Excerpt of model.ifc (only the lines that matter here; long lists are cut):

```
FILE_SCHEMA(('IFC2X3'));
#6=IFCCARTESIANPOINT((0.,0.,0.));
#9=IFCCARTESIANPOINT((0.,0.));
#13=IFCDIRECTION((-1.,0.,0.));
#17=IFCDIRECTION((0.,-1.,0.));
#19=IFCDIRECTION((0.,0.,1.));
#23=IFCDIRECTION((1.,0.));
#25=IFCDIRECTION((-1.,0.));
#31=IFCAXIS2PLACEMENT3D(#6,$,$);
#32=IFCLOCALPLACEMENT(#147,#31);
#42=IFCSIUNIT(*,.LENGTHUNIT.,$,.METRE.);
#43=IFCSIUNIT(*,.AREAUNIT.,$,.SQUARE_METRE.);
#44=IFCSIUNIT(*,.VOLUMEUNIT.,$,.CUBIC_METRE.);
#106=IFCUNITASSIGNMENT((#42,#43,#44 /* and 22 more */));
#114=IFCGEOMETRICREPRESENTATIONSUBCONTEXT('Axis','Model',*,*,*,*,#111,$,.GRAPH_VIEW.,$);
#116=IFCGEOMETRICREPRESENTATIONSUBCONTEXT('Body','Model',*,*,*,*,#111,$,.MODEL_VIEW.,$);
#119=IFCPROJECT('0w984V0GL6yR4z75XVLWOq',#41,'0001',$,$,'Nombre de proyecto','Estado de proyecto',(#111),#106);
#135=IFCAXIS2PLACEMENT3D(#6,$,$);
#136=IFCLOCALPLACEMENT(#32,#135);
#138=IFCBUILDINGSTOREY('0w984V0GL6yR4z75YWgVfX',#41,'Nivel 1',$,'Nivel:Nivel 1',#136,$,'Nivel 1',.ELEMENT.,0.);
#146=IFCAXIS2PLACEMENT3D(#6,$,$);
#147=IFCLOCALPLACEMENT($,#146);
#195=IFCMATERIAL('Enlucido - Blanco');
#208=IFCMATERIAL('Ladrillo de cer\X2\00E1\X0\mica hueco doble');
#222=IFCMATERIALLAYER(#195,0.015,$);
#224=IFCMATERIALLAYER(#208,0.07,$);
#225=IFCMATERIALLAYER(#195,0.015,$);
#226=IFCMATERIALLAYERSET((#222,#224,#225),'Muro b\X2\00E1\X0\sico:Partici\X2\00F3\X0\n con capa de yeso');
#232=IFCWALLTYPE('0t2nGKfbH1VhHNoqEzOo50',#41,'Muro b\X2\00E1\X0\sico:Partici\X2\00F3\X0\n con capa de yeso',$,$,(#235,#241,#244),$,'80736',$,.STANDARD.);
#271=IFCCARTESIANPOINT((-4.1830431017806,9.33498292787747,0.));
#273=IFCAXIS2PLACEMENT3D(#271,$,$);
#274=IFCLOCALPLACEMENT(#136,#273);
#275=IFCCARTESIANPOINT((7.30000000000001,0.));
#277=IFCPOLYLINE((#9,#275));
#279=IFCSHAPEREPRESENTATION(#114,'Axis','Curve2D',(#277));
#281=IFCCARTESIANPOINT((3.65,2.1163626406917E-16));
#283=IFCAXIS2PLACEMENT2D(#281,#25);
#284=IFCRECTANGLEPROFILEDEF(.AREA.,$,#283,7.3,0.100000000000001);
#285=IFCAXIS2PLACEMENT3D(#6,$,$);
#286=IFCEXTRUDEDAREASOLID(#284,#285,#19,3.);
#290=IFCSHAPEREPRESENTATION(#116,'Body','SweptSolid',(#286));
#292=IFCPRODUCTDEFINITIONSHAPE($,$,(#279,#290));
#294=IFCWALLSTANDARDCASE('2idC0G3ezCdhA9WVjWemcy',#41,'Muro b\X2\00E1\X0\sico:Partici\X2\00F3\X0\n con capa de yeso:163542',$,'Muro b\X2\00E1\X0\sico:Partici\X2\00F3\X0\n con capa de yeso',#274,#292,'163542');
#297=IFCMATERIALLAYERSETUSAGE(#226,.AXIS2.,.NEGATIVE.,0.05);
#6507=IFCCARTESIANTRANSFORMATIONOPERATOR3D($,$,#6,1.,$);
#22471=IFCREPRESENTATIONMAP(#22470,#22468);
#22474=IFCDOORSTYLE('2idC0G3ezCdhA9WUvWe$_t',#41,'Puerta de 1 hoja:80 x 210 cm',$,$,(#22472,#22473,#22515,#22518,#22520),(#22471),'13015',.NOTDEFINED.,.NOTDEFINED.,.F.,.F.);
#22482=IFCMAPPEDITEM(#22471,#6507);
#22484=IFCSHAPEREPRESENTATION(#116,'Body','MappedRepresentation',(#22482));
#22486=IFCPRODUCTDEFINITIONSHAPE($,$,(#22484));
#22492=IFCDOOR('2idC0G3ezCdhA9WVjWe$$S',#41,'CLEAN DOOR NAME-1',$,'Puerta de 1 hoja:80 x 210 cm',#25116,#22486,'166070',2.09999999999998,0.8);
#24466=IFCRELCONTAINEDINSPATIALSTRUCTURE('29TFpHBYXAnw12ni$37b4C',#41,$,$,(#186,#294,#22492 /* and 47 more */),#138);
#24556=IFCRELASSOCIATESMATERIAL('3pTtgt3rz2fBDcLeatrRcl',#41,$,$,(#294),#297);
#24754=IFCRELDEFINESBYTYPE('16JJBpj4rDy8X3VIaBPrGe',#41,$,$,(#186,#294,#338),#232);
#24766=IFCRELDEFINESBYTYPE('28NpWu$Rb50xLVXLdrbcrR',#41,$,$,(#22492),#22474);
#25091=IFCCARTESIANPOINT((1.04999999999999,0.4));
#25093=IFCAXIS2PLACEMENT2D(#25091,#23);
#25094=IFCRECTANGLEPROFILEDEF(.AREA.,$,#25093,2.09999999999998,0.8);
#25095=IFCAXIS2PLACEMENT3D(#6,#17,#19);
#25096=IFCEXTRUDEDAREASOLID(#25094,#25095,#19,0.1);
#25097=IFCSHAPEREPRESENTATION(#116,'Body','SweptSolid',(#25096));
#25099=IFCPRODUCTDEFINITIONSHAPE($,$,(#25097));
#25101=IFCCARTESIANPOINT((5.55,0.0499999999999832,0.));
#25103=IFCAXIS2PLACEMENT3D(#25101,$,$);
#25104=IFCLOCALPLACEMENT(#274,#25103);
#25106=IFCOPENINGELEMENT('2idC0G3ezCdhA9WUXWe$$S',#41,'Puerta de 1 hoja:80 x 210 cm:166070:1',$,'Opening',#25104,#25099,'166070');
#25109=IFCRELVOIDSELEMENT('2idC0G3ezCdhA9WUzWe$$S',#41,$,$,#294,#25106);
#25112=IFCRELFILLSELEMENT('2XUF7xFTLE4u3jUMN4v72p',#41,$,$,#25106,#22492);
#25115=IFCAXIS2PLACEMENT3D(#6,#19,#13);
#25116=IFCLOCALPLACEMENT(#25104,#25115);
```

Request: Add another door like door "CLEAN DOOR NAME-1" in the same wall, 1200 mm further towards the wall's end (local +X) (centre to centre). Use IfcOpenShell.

```python
import ifcopenshell
import ifcopenshell.api.feature
import ifcopenshell.api.geometry
import ifcopenshell.api.root
import ifcopenshell.geom
import ifcopenshell.util.element
import ifcopenshell.util.placement
import ifcopenshell.util.shape
import ifcopenshell.util.unit

model = ifcopenshell.open("model.ifc")
unit_scale = ifcopenshell.util.unit.calculate_unit_scale(model)
settings = ifcopenshell.geom.settings()


def volume(element):
    """Net volume in cubic metres, openings subtracted."""
    shape = ifcopenshell.geom.create_shape(settings, element)
    return ifcopenshell.util.shape.get_volume(shape.geometry)


def reuse_history(source, copy):
    """copy_class also copies each property set's owner history, people and application; keep the originals."""
    for rel in copy.IsDefinedBy:
        if rel.is_a("IfcRelDefinesByProperties") and (history := rel.RelatingPropertyDefinition.OwnerHistory):
            rel.RelatingPropertyDefinition.OwnerHistory = source.OwnerHistory
            ifcopenshell.util.element.remove_deep2(model, history)


door = model.by_guid("2idC0G3ezCdhA9WVjWe$$S")
opening = door.FillsVoids[0].RelatingOpeningElement
wall = opening.VoidsElements[0].RelatingBuildingElement
before = volume(wall)
shift = ifcopenshell.util.placement.get_local_placement(wall.ObjectPlacement)[:3, 0] * 1.2 / unit_scale

# copy_class copies the void relationship, type, container and properties, but no geometry.
new_opening = ifcopenshell.api.root.copy_class(model, product=opening)
new_opening.Representation = ifcopenshell.util.element.copy_deep(
    model, opening.Representation, exclude=["IfcGeometricRepresentationContext", "IfcRepresentationMap"]
)
new_opening.Name = "Puerta de 1 hoja:80 x 210 cm"
new_opening.Tag = None
new_door = ifcopenshell.api.root.copy_class(model, product=door)
new_door.Representation = ifcopenshell.util.element.copy_deep(
    model, door.Representation, exclude=["IfcGeometricRepresentationContext", "IfcRepresentationMap"]
)
new_door.Tag = None
reuse_history(door, new_door)
fills = ifcopenshell.api.feature.add_filling(model, opening=new_opening, element=new_door)
fills.OwnerHistory = new_door.OwnerHistory  # required in IFC2X3

for old, new in ((opening, new_opening), (door, new_door)):
    matrix = ifcopenshell.util.placement.get_local_placement(old.ObjectPlacement)
    matrix[:3, 3] += shift
    ifcopenshell.api.geometry.edit_object_placement(model, product=new, matrix=matrix, is_si=False)

after = volume(wall)

print(f"wall volume {before:.3f} -> {after:.3f} m3")

model.write("model-out.ifc")
```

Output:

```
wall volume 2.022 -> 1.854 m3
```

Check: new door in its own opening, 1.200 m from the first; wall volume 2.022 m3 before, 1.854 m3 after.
